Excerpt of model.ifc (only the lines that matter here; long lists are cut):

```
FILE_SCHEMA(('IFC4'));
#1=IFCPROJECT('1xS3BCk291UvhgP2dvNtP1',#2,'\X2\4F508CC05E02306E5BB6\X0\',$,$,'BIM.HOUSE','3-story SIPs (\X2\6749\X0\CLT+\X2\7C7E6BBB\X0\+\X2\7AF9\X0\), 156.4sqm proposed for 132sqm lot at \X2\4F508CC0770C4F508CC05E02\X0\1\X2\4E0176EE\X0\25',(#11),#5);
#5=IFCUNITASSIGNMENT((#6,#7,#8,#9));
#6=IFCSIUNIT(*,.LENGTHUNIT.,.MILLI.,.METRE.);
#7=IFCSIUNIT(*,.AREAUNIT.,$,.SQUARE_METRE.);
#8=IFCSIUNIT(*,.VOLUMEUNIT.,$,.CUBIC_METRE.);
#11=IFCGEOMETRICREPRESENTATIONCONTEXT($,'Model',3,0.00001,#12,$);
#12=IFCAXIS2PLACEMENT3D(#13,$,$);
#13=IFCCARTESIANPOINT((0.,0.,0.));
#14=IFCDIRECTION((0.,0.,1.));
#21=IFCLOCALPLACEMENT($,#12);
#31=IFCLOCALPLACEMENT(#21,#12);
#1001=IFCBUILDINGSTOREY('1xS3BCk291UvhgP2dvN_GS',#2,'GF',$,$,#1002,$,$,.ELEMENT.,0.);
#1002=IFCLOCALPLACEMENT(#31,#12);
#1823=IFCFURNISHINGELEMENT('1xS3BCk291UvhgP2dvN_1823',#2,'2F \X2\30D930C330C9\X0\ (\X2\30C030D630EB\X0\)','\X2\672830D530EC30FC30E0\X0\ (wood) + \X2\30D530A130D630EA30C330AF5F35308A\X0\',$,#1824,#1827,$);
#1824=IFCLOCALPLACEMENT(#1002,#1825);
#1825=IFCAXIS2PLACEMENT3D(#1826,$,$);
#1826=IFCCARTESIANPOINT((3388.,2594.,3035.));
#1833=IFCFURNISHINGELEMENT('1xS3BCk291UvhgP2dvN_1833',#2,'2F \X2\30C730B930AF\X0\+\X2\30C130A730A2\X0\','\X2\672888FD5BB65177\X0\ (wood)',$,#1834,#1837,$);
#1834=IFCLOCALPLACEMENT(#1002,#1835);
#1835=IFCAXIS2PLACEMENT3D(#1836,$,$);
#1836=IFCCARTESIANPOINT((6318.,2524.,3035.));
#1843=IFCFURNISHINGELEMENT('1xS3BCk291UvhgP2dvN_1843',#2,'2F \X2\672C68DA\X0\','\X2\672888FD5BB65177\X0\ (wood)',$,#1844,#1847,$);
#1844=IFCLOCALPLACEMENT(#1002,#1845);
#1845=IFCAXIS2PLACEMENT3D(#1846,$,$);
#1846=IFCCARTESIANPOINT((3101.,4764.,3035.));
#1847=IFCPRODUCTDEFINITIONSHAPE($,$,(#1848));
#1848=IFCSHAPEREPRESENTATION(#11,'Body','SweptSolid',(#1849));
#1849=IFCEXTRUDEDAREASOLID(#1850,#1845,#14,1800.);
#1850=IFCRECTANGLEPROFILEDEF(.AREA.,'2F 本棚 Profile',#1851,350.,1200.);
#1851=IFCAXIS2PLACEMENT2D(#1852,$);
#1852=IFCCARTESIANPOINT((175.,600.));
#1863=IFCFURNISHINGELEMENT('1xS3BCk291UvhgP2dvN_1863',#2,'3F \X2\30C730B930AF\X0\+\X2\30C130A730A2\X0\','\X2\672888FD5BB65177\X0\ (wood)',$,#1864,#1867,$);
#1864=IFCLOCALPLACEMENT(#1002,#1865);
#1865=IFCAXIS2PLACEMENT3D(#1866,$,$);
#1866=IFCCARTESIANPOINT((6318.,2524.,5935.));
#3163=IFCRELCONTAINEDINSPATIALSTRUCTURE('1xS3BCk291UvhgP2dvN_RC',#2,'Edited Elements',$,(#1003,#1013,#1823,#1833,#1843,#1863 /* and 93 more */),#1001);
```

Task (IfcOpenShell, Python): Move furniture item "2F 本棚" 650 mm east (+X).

```python
import ifcopenshell
import ifcopenshell.api.geometry
import ifcopenshell.util.placement

model = ifcopenshell.open("model.ifc")

item = model.by_guid("1xS3BCk291UvhgP2dvN_1843")
matrix = ifcopenshell.util.placement.get_local_placement(item.ObjectPlacement)
matrix[0, 3] += 650.0
ifcopenshell.api.geometry.edit_object_placement(model, product=item, matrix=matrix, is_si=False)

print(ifcopenshell.util.placement.get_local_placement(item.ObjectPlacement).round(3) + 0.0)

model.write("model_edited.ifc")
```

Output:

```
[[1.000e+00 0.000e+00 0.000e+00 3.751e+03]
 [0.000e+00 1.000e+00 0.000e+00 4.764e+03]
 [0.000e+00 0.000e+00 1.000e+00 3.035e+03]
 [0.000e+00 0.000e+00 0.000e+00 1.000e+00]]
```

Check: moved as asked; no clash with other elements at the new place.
